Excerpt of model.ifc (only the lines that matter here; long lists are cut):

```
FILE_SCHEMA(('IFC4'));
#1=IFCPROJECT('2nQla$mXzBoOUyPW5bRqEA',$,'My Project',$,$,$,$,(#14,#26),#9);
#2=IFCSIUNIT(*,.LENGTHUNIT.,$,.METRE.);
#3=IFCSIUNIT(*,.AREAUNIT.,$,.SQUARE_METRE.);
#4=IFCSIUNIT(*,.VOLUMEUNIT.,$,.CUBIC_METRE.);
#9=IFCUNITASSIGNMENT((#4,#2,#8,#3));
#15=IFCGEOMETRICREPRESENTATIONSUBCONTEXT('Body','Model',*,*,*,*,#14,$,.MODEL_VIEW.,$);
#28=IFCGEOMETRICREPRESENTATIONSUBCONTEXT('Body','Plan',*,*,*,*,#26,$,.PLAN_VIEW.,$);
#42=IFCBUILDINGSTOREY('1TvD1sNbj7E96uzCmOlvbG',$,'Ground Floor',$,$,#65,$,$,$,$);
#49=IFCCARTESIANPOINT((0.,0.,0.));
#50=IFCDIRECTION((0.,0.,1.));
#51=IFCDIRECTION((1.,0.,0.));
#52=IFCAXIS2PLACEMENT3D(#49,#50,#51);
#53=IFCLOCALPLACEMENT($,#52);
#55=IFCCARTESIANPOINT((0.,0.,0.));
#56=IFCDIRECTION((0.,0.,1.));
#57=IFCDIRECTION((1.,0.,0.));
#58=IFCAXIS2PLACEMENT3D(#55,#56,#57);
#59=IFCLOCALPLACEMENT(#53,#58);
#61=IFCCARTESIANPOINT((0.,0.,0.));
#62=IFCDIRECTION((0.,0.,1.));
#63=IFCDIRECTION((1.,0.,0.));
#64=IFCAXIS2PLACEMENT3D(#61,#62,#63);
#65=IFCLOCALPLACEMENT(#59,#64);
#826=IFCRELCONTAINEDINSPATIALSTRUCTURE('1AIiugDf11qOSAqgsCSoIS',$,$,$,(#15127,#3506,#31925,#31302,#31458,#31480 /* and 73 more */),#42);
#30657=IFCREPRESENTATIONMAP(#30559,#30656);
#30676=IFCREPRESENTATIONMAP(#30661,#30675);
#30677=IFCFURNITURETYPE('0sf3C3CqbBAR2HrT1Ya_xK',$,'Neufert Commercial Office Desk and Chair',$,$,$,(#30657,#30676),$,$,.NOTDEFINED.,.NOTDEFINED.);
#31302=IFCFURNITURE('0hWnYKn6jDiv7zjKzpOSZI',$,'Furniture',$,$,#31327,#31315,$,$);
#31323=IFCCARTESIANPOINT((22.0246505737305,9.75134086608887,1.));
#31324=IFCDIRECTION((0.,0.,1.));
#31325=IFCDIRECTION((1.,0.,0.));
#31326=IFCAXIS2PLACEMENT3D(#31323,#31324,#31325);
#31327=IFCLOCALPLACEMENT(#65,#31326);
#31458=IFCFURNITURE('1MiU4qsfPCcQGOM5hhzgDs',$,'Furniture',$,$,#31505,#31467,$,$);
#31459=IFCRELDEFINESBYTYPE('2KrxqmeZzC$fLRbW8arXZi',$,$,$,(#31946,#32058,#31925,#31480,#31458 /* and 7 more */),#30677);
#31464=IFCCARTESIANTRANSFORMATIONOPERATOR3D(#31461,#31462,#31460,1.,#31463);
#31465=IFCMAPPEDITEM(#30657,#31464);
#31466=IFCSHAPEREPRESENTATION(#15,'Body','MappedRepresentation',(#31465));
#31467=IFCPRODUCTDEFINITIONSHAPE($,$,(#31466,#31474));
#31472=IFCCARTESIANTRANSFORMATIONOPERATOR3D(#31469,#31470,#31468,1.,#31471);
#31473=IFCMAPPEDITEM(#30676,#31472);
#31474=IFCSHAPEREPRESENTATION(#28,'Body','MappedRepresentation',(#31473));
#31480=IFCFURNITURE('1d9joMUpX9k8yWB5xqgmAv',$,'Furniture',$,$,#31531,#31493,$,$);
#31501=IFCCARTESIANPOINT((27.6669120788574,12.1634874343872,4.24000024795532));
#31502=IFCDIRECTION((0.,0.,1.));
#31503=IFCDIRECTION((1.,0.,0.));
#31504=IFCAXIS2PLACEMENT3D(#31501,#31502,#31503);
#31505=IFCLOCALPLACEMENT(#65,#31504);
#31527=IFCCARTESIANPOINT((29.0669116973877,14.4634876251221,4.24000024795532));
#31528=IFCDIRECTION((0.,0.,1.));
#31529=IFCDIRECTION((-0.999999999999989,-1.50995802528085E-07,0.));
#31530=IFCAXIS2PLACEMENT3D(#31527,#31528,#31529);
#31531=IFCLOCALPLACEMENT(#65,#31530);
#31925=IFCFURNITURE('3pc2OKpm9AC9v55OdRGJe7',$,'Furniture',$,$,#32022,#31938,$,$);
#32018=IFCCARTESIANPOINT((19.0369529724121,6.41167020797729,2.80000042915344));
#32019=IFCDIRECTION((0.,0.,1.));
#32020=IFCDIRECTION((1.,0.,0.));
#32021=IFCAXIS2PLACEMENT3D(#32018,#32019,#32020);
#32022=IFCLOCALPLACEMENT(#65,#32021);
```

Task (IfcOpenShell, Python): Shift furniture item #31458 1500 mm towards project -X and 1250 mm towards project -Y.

```python
import ifcopenshell
import ifcopenshell.api.geometry
import ifcopenshell.util.placement

model = ifcopenshell.open("model.ifc")

item = model.by_guid("1MiU4qsfPCcQGOM5hhzgDs")
matrix = ifcopenshell.util.placement.get_local_placement(item.ObjectPlacement)
matrix[0, 3] -= 1.5
matrix[1, 3] -= 1.25
ifcopenshell.api.geometry.edit_object_placement(model, product=item, matrix=matrix, is_si=False)

print(ifcopenshell.util.placement.get_local_placement(item.ObjectPlacement).round(3) + 0.0)

model.write("model_edited.ifc")
```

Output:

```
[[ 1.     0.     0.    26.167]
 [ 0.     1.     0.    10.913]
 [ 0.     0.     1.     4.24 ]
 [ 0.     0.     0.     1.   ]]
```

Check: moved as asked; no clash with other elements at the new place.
